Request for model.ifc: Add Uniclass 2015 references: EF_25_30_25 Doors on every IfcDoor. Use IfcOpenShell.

First a look at what the model holds.

```python
import ifcopenshell

model = ifcopenshell.open("model.ifc")
print(model.schema)
print("classifications:", [c.Name for c in model.by_type("IfcClassification")])
for ifc_class in ("IfcDoor", "IfcRoof", "IfcStair", "IfcWall", "IfcWindow"):
    print(ifc_class, len(model.by_type(ifc_class)))
```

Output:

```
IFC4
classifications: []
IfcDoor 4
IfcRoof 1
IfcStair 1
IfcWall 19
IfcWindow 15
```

```python
import ifcopenshell
import ifcopenshell.api.classification

model = ifcopenshell.open("model.ifc")

system = ifcopenshell.api.classification.add_classification(model, classification="Uniclass 2015")

codes = {
    "IfcDoor": ("EF_25_30_25", "Doors"),
}
for ifc_class, (code, name) in codes.items():
    products = model.by_type(ifc_class)
    ifcopenshell.api.classification.add_reference(
        model, products=products, classification=system, identification=code, name=name
    )
    print(code, len(products))

model.write("model-out.ifc")
```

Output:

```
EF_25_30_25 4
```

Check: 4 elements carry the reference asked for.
